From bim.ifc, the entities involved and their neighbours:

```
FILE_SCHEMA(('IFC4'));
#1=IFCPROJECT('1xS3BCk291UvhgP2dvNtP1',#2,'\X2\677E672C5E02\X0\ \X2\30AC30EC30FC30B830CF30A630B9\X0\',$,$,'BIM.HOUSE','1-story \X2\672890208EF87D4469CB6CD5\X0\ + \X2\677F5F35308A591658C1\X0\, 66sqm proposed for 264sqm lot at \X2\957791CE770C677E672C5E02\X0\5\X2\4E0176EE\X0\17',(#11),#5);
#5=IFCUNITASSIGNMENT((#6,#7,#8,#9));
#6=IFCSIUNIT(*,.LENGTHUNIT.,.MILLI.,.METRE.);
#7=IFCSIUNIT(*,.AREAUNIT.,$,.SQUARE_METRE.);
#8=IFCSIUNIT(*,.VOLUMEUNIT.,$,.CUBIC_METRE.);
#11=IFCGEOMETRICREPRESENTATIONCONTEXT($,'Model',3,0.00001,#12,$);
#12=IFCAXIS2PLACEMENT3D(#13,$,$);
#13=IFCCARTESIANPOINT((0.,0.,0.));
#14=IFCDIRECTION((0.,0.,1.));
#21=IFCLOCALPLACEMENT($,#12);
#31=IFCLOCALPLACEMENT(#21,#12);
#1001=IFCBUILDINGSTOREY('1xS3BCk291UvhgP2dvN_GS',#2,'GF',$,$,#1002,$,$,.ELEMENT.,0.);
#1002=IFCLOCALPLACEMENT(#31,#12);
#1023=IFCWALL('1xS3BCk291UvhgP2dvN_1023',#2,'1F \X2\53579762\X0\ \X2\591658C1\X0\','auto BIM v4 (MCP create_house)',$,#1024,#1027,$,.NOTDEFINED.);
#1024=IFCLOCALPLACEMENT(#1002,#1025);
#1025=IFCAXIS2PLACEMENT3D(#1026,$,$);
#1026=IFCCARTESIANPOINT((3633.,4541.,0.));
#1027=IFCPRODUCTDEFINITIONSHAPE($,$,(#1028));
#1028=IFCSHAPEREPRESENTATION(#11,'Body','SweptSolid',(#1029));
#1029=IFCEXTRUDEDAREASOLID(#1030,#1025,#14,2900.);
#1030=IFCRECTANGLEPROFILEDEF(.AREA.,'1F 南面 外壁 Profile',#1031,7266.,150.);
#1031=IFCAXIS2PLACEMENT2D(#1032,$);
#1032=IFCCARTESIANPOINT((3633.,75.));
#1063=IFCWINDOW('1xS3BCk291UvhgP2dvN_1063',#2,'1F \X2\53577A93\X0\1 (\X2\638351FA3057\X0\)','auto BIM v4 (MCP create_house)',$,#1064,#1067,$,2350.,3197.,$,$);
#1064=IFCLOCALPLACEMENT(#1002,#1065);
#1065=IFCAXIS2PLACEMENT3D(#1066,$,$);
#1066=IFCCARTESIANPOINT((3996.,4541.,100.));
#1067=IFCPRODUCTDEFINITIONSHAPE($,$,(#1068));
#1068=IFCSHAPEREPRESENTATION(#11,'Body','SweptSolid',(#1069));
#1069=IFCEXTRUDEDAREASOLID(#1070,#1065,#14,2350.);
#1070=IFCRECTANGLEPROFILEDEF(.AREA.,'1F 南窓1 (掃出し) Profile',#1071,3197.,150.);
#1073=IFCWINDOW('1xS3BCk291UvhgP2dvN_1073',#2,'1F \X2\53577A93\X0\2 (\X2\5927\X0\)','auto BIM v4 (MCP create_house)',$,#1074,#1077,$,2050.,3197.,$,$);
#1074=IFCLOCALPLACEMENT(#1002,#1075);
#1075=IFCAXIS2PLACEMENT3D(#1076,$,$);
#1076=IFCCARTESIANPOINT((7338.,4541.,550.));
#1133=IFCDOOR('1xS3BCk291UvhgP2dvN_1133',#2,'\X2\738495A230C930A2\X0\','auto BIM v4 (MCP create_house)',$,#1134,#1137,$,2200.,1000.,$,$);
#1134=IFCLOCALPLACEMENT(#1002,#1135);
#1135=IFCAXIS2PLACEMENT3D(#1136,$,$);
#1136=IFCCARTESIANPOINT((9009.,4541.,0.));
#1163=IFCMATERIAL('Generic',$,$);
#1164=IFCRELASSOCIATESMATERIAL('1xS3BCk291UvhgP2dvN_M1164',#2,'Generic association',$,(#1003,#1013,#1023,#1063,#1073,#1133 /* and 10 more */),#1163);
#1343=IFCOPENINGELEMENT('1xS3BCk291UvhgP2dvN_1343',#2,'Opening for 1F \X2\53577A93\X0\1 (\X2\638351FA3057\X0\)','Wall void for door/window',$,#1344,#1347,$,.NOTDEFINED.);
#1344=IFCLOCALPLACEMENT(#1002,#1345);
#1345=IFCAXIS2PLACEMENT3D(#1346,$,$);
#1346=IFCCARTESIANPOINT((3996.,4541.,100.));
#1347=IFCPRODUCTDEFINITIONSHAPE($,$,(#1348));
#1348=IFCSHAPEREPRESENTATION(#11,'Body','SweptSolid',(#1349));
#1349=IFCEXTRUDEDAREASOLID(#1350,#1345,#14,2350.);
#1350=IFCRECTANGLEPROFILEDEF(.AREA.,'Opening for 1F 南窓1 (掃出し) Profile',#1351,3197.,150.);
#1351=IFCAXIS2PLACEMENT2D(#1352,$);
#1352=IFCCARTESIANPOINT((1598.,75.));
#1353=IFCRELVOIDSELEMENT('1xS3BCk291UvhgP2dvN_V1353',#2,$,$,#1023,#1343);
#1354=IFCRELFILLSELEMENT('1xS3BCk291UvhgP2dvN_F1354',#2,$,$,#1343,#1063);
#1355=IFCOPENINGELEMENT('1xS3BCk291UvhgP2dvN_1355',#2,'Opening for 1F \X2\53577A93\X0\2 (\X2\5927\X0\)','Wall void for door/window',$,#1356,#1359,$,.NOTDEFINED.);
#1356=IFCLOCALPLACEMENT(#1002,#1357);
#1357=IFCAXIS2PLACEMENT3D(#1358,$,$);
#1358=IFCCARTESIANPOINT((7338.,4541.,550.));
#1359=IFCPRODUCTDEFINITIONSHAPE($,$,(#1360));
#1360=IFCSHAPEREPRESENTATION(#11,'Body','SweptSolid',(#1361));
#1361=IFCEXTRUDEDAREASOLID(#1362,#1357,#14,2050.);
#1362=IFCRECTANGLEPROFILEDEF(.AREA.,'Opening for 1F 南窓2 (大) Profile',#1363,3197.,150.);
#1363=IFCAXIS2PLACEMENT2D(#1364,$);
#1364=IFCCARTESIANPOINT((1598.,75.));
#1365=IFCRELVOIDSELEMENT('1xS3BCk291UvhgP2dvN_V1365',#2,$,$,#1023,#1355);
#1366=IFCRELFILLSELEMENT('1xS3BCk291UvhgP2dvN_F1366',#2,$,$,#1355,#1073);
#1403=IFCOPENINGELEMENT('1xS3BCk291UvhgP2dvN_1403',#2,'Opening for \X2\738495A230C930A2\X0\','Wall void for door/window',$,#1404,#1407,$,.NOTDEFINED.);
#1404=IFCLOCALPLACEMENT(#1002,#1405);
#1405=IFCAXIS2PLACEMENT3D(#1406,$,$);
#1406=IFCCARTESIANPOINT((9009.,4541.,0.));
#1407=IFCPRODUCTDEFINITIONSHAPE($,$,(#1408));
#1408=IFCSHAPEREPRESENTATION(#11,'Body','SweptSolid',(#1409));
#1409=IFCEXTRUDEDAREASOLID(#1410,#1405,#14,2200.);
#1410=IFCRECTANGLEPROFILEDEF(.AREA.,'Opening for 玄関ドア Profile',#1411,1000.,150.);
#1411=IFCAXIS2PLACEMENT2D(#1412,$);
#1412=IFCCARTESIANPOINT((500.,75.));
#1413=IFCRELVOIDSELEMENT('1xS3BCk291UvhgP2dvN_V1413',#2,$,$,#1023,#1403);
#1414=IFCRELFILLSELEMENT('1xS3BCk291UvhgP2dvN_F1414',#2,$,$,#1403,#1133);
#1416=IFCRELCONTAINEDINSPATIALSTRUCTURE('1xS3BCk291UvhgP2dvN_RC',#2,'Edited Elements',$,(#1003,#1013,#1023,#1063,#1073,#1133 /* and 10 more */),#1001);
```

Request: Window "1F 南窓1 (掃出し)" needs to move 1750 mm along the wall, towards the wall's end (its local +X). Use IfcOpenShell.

```python
import ifcopenshell
import ifcopenshell.api.geometry
import ifcopenshell.util.placement
import ifcopenshell.util.unit

model = ifcopenshell.open("bim.ifc")
unit_scale = ifcopenshell.util.unit.calculate_unit_scale(model)

window = model.by_guid("1xS3BCk291UvhgP2dvN_1063")
opening = window.FillsVoids[0].RelatingOpeningElement
wall = opening.VoidsElements[0].RelatingBuildingElement

wall_matrix = ifcopenshell.util.placement.get_local_placement(wall.ObjectPlacement)
shift = wall_matrix[:3, 0] * 1.75 / unit_scale
before = ifcopenshell.util.placement.get_local_placement(window.ObjectPlacement)[:3, 3].copy()

# The window is not placed relative to its opening, so move both.
for product in (opening, window):
    matrix = ifcopenshell.util.placement.get_local_placement(product.ObjectPlacement)
    matrix[:3, 3] += shift
    ifcopenshell.api.geometry.edit_object_placement(model, product=product, matrix=matrix, is_si=False)

after = ifcopenshell.util.placement.get_local_placement(window.ObjectPlacement)[:3, 3]
print("window moved by", (after - before).round(3) + 0.0)

model.write("bim_v2.ifc")
```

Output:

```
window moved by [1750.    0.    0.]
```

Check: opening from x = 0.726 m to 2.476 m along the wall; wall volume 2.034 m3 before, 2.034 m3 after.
